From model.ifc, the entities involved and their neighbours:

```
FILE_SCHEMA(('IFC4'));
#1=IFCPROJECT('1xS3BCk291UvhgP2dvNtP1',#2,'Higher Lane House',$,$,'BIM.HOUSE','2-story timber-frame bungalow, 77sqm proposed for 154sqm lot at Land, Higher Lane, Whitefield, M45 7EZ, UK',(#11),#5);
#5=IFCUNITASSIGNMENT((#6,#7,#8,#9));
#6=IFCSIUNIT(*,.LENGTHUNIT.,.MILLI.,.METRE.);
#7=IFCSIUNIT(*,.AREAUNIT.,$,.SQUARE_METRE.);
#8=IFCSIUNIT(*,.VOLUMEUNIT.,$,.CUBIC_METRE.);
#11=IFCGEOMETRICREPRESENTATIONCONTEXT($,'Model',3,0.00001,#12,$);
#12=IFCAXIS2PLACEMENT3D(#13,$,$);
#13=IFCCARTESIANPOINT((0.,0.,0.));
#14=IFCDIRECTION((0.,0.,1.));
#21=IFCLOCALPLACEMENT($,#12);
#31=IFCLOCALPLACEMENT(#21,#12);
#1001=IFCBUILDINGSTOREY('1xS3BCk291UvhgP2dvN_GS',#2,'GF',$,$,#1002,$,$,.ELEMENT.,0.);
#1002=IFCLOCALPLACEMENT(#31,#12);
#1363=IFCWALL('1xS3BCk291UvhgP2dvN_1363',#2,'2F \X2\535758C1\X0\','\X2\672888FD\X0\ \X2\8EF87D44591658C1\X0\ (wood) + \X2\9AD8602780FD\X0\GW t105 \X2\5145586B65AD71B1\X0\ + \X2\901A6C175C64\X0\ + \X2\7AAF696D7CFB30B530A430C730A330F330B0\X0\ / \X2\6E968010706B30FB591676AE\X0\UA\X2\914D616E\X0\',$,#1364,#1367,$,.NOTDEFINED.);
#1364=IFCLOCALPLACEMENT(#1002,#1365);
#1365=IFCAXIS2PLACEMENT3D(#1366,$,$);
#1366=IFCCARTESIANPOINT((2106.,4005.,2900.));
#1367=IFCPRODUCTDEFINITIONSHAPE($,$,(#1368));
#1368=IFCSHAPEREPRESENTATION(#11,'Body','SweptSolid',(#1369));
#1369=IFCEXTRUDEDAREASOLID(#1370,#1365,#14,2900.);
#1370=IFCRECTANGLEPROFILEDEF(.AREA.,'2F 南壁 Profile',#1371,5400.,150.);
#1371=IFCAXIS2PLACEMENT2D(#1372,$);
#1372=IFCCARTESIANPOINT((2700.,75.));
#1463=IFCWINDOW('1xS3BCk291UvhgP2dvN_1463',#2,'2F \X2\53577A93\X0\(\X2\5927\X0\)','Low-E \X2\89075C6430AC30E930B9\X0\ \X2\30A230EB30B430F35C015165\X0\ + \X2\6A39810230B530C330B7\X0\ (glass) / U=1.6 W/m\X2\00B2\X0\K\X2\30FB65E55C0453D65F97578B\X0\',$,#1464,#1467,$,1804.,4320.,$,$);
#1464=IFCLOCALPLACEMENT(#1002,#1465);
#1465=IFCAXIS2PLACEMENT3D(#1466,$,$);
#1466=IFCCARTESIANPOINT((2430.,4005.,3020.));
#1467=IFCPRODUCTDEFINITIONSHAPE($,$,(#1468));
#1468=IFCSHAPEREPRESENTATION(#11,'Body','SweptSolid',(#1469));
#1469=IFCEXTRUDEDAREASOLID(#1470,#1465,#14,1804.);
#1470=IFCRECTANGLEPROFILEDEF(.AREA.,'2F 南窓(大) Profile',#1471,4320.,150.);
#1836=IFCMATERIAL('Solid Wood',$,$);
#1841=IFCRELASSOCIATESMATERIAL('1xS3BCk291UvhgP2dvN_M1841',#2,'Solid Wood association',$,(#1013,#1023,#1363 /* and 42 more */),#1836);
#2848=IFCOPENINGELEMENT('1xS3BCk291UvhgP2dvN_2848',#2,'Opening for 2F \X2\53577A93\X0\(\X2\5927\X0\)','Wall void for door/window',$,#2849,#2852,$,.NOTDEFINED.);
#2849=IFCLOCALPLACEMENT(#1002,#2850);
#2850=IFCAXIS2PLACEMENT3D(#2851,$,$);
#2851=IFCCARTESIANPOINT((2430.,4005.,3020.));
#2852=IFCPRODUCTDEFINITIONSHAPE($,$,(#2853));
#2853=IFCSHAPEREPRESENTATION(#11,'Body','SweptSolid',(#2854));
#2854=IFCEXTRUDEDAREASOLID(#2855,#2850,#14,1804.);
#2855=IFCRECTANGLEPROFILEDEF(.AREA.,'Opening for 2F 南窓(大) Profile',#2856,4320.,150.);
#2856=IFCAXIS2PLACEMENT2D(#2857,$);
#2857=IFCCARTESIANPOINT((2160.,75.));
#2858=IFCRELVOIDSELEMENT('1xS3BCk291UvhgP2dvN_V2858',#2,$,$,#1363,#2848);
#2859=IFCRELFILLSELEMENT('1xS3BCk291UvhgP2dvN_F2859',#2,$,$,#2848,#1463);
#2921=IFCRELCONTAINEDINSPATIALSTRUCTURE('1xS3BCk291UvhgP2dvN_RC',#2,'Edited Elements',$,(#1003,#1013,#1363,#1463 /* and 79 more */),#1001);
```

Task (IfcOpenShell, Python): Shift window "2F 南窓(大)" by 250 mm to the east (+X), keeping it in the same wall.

```python
import ifcopenshell
import ifcopenshell.api.geometry
import ifcopenshell.util.placement
import ifcopenshell.util.unit

model = ifcopenshell.open("model.ifc")
unit_scale = ifcopenshell.util.unit.calculate_unit_scale(model)

window = model.by_guid("1xS3BCk291UvhgP2dvN_1463")
opening = window.FillsVoids[0].RelatingOpeningElement
wall = opening.VoidsElements[0].RelatingBuildingElement

wall_matrix = ifcopenshell.util.placement.get_local_placement(wall.ObjectPlacement)
shift = wall_matrix[:3, 0] * 0.25 / unit_scale
before = ifcopenshell.util.placement.get_local_placement(window.ObjectPlacement)[:3, 3].copy()

# The window is not placed relative to its opening, so move both.
for product in (opening, window):
    matrix = ifcopenshell.util.placement.get_local_placement(product.ObjectPlacement)
    matrix[:3, 3] += shift
    ifcopenshell.api.geometry.edit_object_placement(model, product=product, matrix=matrix, is_si=False)

after = ifcopenshell.util.placement.get_local_placement(window.ObjectPlacement)[:3, 3]
print("window moved by", (after - before).round(3) + 0.0)

model.write("model_v2.ifc")
```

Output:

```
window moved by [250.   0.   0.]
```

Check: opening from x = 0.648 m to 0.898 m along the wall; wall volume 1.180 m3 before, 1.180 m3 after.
